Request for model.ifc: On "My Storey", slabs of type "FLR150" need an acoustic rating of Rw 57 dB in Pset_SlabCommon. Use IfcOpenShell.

First a look at what the model holds.

```python
import ifcopenshell
import ifcopenshell.util.element

model = ifcopenshell.open("model.ifc")
print(model.schema)
storey = next(s for s in model.by_type("IfcBuildingStorey") if s.Name == "My Storey")
slabs = [e for e in ifcopenshell.util.element.get_decomposition(storey) if e.is_a("IfcSlab")]
seen = {}
for e in slabs:
    element_type = ifcopenshell.util.element.get_type(e)
    key = (element_type.Name if element_type != e and element_type else None, ifcopenshell.util.element.get_pset(e, "Pset_SlabCommon", "AcousticRating"))
    seen[key] = seen.get(key, 0) + 1
for (name, value), count in sorted(seen.items(), key=str):
    print(count, "x", name, "|", value)
```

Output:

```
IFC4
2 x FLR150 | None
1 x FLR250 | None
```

```python
import ifcopenshell
import ifcopenshell.api.pset
import ifcopenshell.util.element

model = ifcopenshell.open("model.ifc")

storey = next(s for s in model.by_type("IfcBuildingStorey") if s.Name == "My Storey")
slabs = [e for e in ifcopenshell.util.element.get_decomposition(storey) if e.is_a("IfcSlab")]

count = 0
for e in slabs:
    element_type = ifcopenshell.util.element.get_type(e)
    if element_type in (None, e) or element_type.Name != "FLR150":
        continue
    # add_pset returns the element's existing set when there is one.
    pset = ifcopenshell.api.pset.add_pset(model, product=e, name="Pset_SlabCommon")
    ifcopenshell.api.pset.edit_pset(model, pset=pset, properties={"AcousticRating": "Rw 57 dB"})
    count += 1

print(count, "slabs updated")

model.write("model_rev.ifc")
```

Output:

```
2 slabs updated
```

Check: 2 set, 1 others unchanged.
